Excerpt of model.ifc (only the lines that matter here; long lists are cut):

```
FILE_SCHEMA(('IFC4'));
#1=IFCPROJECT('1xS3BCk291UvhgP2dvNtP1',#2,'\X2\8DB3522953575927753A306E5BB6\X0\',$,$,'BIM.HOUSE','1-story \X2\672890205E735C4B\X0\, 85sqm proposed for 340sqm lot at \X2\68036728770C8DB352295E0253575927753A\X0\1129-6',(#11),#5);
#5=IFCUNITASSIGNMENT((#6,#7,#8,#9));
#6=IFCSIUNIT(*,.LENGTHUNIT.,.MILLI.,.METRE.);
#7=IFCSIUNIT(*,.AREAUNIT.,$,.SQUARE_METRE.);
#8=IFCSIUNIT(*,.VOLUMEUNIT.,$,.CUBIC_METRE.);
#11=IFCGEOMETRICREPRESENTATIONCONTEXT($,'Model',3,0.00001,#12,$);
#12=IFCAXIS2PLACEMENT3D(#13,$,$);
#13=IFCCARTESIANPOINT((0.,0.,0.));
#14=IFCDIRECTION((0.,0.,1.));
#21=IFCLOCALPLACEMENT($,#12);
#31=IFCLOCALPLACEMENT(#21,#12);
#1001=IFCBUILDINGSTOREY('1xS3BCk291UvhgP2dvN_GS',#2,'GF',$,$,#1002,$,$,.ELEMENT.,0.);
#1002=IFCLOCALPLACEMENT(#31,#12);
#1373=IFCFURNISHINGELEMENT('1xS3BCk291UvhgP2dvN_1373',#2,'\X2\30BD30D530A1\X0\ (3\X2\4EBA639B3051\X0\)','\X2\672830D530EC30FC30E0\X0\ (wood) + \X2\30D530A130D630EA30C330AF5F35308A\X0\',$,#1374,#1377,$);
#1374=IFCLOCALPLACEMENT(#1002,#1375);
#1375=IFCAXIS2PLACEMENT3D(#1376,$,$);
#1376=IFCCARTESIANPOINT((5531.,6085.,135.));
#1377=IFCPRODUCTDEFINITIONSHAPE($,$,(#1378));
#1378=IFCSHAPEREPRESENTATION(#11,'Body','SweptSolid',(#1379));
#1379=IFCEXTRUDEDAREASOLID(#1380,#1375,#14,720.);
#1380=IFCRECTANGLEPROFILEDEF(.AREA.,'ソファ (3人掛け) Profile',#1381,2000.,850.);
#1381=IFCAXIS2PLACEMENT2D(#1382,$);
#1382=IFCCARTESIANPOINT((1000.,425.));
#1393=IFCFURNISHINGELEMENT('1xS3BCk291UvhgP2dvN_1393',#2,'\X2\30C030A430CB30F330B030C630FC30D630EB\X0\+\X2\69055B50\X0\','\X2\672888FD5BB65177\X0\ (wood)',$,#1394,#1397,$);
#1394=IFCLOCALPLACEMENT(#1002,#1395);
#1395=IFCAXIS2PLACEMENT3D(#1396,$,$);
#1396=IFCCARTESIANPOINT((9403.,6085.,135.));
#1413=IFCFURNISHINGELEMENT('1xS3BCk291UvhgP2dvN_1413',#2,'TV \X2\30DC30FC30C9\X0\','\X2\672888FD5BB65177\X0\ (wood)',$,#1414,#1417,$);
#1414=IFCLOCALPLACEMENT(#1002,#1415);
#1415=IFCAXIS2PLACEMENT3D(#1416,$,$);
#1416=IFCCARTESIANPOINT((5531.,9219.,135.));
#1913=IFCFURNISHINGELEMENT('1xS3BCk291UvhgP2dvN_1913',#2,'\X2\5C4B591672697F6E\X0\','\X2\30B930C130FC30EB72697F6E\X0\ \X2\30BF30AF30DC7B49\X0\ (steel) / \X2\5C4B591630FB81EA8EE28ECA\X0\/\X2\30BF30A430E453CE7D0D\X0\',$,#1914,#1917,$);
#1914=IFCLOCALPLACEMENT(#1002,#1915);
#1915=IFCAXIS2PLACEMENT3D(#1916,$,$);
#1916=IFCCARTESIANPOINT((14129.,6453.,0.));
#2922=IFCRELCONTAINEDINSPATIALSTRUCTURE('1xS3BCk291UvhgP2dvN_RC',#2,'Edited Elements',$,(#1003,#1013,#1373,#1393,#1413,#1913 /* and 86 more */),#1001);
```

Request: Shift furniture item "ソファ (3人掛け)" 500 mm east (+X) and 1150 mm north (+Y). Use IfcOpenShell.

```python
import ifcopenshell
import ifcopenshell.api.geometry
import ifcopenshell.util.placement

model = ifcopenshell.open("model.ifc")

item = model.by_guid("1xS3BCk291UvhgP2dvN_1373")
matrix = ifcopenshell.util.placement.get_local_placement(item.ObjectPlacement)
matrix[0, 3] += 500.0
matrix[1, 3] += 1150.0
ifcopenshell.api.geometry.edit_object_placement(model, product=item, matrix=matrix, is_si=False)

print(ifcopenshell.util.placement.get_local_placement(item.ObjectPlacement).round(3) + 0.0)

model.write("model_rev.ifc")
```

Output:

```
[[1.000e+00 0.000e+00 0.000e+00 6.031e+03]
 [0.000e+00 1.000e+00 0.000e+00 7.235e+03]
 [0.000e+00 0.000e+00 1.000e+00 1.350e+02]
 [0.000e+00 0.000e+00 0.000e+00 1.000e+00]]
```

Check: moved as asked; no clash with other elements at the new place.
